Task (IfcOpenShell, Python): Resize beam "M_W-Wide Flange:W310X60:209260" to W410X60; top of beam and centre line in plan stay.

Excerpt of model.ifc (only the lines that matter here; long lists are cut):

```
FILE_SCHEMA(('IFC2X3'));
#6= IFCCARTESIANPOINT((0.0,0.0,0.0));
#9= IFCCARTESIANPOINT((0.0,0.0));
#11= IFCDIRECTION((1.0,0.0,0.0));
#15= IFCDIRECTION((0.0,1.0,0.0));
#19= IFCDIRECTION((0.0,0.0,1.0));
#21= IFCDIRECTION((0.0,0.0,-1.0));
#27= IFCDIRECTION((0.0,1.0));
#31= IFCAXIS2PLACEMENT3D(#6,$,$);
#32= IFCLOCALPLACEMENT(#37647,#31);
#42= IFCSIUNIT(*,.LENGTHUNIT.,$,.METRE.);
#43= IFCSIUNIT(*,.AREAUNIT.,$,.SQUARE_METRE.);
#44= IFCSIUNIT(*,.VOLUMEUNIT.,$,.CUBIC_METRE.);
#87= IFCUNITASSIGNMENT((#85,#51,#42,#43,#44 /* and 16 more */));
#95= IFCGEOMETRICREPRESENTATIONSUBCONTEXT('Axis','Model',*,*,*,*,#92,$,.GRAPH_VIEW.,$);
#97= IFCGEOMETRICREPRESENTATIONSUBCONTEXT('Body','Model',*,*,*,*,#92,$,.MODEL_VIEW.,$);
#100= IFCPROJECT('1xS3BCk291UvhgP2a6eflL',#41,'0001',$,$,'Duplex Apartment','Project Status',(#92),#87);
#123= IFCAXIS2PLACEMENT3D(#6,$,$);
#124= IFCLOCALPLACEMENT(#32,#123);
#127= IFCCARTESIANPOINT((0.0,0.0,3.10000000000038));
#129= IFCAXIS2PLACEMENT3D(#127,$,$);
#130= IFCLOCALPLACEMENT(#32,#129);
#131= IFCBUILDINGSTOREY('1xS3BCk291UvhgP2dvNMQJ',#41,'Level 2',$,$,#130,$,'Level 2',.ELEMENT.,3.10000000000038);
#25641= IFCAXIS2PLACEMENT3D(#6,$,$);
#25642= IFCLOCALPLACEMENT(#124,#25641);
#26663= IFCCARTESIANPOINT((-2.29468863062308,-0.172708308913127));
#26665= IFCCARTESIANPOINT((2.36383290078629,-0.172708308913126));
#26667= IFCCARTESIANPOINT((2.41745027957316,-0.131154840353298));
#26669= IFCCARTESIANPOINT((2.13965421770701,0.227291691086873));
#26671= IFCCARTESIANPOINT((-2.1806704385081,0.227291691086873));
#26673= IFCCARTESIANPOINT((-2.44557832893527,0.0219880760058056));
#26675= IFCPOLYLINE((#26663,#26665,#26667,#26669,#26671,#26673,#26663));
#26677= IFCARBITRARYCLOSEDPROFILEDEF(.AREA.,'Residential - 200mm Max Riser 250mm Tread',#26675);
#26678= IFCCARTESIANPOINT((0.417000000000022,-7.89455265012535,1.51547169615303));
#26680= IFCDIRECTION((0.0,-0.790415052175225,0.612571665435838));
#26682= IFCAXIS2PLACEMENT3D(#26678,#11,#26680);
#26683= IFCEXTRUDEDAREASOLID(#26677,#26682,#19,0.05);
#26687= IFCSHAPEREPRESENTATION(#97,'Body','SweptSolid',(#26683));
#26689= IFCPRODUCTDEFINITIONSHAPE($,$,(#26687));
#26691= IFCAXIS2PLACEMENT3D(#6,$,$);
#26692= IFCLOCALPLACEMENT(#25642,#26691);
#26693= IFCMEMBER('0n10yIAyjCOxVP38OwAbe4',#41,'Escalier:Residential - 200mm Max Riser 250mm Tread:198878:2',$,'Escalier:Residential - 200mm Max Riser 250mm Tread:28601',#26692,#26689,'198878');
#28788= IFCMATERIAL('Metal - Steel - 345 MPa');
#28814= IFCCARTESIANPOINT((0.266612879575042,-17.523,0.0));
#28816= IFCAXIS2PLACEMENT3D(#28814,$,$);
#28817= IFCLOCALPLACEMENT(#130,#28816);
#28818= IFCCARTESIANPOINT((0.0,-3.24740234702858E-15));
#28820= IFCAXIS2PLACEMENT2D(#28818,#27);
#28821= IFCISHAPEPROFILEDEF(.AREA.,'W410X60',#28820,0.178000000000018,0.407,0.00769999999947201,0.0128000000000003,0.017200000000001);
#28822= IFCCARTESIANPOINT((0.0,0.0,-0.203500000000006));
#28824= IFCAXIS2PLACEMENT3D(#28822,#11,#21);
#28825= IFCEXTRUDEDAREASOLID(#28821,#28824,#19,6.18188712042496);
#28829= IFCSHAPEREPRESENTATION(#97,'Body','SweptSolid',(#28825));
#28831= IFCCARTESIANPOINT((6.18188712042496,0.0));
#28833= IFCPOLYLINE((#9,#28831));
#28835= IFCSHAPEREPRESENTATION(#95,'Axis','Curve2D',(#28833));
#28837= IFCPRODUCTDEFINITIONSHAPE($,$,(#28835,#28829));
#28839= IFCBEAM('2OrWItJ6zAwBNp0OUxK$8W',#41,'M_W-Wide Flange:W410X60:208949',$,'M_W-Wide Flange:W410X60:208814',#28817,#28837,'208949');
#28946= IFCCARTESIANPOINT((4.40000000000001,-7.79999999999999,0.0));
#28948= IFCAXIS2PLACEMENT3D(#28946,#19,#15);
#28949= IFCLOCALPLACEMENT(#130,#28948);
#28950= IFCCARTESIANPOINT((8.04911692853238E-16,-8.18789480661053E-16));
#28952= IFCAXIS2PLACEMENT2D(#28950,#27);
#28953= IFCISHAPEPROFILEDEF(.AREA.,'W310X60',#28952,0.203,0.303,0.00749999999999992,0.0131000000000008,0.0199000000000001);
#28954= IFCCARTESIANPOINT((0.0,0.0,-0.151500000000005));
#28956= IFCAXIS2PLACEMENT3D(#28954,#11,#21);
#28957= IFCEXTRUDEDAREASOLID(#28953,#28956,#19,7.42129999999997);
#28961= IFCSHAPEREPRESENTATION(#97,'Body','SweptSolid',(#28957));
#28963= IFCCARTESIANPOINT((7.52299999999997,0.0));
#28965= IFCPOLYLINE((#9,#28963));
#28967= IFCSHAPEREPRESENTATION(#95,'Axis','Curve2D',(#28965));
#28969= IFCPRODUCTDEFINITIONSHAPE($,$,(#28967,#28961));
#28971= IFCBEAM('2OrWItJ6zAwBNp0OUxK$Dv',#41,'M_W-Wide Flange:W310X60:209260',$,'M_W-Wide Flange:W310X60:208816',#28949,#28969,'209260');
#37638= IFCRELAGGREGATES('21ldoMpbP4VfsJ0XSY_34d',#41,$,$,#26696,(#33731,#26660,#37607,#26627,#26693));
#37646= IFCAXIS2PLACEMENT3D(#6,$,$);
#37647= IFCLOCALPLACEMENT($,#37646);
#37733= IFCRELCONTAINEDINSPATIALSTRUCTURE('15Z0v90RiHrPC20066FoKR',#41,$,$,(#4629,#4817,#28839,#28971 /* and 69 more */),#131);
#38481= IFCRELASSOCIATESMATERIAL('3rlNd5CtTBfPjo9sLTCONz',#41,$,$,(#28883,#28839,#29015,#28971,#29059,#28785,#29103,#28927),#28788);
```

```python
import ifcopenshell
import ifcopenshell.util.element
import ifcopenshell.util.representation

model = ifcopenshell.open("model.ifc")

member = model.by_guid("2OrWItJ6zAwBNp0OUxK$Dv")
source = next(p for p in model.by_type("IfcIShapeProfileDef") if p.ProfileName == "W410X60")

body = ifcopenshell.util.representation.get_representation(member, "Model", "Body")
solid = body.Items[0]
old_profile = solid.SweptArea

# Copy the section's sizes but keep this member's own profile position.
profile = ifcopenshell.util.element.copy(model, source)
# Profiles are centred, so shift by half the change in depth to hold the top.
shift = (old_profile.OverallDepth - profile.OverallDepth) / 2
x, y = old_profile.Position.Location.Coordinates
up = (-1.0, 0.0)  # upwards, in the solid's own plane
location = model.createIfcCartesianPoint((x + up[0] * shift, y + up[1] * shift))
profile.Position = model.createIfcAxis2Placement2D(location, old_profile.Position.RefDirection)
solid.SweptArea = profile
if not model.get_total_inverses(old_profile):
    ifcopenshell.util.element.remove_deep2(model, old_profile)
member.Name = member.Name.replace("W310X60", "W410X60")
member.ObjectType = member.ObjectType.replace("W310X60", "W410X60")

print(solid.SweptArea)

model.write("model_edited.ifc")
```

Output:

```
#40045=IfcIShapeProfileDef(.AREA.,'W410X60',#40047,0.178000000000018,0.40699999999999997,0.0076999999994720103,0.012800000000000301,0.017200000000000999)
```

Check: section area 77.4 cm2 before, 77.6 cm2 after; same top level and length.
